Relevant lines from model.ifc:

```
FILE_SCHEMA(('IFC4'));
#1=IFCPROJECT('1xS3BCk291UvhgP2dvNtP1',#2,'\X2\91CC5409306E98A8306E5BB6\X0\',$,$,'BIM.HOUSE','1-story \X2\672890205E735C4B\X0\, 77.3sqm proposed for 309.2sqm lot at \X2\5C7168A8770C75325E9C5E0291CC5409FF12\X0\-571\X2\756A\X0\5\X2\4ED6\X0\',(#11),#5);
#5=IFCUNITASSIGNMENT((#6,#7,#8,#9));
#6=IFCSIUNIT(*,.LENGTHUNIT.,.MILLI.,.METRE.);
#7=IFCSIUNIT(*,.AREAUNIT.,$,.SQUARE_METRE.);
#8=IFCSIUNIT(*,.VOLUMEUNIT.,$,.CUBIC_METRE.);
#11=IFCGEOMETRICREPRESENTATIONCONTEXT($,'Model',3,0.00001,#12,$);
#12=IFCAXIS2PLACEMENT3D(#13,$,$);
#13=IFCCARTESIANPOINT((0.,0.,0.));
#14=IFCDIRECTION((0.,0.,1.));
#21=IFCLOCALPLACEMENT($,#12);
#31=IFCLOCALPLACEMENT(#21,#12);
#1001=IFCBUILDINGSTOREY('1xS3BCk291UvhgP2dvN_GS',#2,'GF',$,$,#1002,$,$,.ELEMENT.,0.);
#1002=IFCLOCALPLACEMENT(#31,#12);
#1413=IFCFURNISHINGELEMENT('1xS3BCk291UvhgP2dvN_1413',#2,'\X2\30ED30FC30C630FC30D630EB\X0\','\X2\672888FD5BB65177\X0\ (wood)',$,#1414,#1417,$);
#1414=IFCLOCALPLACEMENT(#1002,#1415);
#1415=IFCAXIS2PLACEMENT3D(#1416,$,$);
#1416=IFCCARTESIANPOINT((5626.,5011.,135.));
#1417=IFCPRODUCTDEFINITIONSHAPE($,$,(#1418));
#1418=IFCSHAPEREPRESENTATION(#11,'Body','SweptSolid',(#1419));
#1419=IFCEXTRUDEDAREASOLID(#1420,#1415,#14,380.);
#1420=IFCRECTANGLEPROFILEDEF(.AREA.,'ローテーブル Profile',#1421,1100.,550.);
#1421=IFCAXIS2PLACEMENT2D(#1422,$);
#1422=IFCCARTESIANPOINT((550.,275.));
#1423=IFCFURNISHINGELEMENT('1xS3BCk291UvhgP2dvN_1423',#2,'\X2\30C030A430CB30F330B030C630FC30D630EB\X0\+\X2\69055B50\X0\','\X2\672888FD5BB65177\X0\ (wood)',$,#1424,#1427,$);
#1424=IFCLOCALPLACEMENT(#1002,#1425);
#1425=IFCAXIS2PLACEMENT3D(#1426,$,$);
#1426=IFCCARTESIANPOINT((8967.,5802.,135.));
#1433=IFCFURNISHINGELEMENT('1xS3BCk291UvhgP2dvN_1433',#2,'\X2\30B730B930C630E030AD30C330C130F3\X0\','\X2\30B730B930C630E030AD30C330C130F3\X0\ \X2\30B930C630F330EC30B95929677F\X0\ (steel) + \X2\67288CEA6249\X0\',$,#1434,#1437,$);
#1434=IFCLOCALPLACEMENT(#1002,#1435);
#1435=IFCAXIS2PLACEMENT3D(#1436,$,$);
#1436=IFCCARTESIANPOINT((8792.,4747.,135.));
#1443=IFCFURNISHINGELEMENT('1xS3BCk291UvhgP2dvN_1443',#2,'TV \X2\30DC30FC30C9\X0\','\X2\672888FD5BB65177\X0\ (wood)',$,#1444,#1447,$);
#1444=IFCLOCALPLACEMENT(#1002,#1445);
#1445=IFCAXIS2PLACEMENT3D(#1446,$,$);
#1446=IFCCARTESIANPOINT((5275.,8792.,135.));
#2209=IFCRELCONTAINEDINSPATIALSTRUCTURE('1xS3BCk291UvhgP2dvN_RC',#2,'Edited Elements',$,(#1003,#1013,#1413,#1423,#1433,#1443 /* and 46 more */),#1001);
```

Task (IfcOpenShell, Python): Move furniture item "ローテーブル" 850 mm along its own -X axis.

```python
import ifcopenshell
import ifcopenshell.api.geometry
import ifcopenshell.util.placement
import ifcopenshell.util.unit

model = ifcopenshell.open("model.ifc")
unit_scale = ifcopenshell.util.unit.calculate_unit_scale(model)

item = model.by_id(1413)
matrix = ifcopenshell.util.placement.get_local_placement(item.ObjectPlacement)
matrix[:3, 3] -= matrix[:3, 0] * 0.85 / unit_scale
ifcopenshell.api.geometry.edit_object_placement(model, product=item, matrix=matrix, is_si=False)

print(ifcopenshell.util.placement.get_local_placement(item.ObjectPlacement).round(3) + 0.0)

model.write("model_rev.ifc")
```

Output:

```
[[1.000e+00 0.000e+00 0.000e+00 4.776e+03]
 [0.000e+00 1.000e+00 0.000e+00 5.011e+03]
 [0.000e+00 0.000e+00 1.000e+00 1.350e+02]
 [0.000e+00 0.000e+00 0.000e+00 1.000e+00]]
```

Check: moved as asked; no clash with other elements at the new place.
